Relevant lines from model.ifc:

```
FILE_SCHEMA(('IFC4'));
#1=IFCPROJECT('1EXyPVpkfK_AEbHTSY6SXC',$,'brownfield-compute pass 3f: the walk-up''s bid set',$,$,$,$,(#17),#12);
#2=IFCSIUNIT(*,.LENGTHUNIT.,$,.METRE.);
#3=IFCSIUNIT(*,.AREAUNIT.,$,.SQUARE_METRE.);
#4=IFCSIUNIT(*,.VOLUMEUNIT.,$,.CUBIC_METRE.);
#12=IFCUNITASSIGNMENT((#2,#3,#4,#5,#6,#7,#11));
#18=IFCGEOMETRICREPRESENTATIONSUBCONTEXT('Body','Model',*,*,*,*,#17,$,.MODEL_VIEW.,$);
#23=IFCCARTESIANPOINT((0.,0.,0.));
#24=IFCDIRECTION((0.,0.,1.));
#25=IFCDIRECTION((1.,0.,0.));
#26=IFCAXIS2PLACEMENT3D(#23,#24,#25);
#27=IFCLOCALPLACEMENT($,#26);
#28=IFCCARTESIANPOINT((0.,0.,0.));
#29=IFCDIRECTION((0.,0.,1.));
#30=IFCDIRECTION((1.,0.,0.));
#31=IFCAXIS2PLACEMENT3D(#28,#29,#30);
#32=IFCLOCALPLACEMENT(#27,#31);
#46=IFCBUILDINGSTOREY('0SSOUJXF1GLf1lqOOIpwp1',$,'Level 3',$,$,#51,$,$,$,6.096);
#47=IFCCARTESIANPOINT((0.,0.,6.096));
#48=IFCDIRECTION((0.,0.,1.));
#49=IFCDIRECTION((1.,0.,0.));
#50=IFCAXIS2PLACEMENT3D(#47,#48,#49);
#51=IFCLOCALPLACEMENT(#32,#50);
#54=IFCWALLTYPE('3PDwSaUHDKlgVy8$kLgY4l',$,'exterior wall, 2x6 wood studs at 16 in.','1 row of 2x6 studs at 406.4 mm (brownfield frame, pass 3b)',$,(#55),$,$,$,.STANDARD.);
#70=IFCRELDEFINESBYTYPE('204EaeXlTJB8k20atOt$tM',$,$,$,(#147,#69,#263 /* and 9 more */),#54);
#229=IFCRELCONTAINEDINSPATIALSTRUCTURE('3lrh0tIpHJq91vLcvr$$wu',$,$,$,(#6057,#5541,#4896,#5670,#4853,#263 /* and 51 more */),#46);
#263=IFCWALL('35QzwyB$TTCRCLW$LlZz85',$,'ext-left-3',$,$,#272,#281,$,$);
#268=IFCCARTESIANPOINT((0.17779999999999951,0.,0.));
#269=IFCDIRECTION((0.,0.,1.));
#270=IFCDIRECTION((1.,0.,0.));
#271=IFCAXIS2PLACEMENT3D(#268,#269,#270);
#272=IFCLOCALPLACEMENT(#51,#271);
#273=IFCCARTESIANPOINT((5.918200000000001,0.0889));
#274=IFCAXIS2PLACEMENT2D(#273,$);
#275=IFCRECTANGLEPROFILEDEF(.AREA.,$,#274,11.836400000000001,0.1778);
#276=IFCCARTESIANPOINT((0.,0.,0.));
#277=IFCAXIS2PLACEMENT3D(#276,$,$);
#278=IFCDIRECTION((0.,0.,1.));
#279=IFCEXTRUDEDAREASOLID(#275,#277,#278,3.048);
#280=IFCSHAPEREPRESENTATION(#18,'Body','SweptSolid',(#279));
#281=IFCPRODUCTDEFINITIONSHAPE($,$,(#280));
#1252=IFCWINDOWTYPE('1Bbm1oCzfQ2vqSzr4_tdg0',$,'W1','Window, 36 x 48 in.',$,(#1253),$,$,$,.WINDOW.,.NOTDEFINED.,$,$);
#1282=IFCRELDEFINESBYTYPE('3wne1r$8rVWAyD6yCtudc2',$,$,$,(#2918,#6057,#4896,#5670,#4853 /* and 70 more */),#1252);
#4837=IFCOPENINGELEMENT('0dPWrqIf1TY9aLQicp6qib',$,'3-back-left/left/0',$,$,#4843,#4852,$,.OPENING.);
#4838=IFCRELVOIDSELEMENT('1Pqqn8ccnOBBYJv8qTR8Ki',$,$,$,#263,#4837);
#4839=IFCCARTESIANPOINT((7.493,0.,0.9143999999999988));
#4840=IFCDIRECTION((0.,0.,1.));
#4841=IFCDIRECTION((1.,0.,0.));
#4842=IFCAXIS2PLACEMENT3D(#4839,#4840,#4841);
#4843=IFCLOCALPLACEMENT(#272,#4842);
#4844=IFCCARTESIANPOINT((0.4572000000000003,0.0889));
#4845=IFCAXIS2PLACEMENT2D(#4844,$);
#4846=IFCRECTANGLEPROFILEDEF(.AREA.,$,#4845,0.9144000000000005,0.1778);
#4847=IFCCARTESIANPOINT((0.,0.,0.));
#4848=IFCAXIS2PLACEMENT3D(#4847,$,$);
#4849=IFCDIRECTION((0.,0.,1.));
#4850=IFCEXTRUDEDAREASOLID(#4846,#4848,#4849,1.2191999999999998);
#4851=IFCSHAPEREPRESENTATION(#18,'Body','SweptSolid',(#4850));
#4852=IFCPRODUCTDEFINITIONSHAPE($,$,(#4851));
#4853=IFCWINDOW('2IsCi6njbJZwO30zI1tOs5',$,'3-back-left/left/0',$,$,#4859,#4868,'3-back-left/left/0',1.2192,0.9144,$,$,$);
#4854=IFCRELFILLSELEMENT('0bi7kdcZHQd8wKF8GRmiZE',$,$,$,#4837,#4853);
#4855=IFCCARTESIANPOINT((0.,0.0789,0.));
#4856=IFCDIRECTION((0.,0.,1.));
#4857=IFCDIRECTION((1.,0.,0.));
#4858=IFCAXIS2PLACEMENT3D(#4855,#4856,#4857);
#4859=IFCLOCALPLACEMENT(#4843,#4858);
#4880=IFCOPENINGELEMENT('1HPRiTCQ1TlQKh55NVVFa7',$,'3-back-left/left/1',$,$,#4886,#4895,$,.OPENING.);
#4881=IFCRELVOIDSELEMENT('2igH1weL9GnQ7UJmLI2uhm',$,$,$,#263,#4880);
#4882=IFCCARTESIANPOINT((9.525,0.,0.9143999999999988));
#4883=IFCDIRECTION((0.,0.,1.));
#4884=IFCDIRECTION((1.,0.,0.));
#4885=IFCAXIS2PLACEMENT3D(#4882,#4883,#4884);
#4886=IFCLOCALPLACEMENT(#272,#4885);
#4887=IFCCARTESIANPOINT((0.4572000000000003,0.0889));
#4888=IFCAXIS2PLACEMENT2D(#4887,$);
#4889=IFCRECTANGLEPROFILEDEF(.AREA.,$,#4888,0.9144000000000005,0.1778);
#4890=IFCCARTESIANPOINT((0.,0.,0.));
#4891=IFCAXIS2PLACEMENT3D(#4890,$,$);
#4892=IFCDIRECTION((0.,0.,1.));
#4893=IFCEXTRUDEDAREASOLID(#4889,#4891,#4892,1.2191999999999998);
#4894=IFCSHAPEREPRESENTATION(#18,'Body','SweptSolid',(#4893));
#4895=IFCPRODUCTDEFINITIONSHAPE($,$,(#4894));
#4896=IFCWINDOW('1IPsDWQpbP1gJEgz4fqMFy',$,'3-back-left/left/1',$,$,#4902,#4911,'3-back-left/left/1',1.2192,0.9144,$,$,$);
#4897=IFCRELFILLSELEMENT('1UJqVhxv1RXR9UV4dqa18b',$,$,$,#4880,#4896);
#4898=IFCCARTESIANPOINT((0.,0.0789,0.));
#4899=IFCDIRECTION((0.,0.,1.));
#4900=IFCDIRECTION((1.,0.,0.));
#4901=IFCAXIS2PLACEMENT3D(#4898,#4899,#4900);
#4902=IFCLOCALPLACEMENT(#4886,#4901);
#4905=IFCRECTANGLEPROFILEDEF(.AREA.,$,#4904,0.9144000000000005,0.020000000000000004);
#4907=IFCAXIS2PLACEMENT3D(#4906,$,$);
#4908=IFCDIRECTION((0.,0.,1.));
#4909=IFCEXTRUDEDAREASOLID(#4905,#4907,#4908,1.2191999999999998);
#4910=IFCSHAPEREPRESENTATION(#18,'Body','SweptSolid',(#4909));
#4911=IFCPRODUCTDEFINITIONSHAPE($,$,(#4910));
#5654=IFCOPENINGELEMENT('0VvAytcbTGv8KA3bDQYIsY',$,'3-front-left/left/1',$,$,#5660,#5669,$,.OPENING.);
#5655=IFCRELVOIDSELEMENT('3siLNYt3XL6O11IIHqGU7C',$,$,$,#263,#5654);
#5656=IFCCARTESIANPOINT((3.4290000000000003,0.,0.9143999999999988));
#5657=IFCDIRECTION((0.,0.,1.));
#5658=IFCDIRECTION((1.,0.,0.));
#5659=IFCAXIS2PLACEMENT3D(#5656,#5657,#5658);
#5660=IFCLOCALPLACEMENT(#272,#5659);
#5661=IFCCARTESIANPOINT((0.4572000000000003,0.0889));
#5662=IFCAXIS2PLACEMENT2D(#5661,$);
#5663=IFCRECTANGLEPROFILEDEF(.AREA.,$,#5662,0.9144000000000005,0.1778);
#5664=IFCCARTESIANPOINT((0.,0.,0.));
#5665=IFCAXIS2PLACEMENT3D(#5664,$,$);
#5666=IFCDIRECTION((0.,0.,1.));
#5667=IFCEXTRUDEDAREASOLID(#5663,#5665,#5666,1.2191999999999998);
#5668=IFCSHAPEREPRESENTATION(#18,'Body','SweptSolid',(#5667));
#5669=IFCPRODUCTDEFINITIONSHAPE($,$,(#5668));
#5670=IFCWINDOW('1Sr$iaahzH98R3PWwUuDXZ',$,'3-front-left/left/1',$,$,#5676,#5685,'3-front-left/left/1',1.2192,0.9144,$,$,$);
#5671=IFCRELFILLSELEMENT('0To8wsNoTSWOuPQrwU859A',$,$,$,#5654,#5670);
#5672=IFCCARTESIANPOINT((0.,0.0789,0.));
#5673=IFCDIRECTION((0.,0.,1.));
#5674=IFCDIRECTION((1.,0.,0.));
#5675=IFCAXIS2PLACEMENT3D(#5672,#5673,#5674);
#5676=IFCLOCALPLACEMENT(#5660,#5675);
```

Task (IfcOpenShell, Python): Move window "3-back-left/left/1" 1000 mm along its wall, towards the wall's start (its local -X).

```python
import ifcopenshell
import ifcopenshell.api.geometry
import ifcopenshell.util.placement

model = ifcopenshell.open("model.ifc")

window = model.by_guid("1IPsDWQpbP1gJEgz4fqMFy")
opening = window.FillsVoids[0].RelatingOpeningElement
wall = opening.VoidsElements[0].RelatingBuildingElement

wall_matrix = ifcopenshell.util.placement.get_local_placement(wall.ObjectPlacement)
shift = wall_matrix[:3, 0] * -1.0
before = ifcopenshell.util.placement.get_local_placement(window.ObjectPlacement)[:3, 3].copy()

# The window is placed relative to its opening, so it follows when the opening moves.
matrix = ifcopenshell.util.placement.get_local_placement(opening.ObjectPlacement)
matrix[:3, 3] += shift
ifcopenshell.api.geometry.edit_object_placement(
    model, product=opening, matrix=matrix, is_si=False, should_transform_children=True
)

after = ifcopenshell.util.placement.get_local_placement(window.ObjectPlacement)[:3, 3]
print("window moved by", (after - before).round(3) + 0.0)

model.write("model_edited.ifc")
```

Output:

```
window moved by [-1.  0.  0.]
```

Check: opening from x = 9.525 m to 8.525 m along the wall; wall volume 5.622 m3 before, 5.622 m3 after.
